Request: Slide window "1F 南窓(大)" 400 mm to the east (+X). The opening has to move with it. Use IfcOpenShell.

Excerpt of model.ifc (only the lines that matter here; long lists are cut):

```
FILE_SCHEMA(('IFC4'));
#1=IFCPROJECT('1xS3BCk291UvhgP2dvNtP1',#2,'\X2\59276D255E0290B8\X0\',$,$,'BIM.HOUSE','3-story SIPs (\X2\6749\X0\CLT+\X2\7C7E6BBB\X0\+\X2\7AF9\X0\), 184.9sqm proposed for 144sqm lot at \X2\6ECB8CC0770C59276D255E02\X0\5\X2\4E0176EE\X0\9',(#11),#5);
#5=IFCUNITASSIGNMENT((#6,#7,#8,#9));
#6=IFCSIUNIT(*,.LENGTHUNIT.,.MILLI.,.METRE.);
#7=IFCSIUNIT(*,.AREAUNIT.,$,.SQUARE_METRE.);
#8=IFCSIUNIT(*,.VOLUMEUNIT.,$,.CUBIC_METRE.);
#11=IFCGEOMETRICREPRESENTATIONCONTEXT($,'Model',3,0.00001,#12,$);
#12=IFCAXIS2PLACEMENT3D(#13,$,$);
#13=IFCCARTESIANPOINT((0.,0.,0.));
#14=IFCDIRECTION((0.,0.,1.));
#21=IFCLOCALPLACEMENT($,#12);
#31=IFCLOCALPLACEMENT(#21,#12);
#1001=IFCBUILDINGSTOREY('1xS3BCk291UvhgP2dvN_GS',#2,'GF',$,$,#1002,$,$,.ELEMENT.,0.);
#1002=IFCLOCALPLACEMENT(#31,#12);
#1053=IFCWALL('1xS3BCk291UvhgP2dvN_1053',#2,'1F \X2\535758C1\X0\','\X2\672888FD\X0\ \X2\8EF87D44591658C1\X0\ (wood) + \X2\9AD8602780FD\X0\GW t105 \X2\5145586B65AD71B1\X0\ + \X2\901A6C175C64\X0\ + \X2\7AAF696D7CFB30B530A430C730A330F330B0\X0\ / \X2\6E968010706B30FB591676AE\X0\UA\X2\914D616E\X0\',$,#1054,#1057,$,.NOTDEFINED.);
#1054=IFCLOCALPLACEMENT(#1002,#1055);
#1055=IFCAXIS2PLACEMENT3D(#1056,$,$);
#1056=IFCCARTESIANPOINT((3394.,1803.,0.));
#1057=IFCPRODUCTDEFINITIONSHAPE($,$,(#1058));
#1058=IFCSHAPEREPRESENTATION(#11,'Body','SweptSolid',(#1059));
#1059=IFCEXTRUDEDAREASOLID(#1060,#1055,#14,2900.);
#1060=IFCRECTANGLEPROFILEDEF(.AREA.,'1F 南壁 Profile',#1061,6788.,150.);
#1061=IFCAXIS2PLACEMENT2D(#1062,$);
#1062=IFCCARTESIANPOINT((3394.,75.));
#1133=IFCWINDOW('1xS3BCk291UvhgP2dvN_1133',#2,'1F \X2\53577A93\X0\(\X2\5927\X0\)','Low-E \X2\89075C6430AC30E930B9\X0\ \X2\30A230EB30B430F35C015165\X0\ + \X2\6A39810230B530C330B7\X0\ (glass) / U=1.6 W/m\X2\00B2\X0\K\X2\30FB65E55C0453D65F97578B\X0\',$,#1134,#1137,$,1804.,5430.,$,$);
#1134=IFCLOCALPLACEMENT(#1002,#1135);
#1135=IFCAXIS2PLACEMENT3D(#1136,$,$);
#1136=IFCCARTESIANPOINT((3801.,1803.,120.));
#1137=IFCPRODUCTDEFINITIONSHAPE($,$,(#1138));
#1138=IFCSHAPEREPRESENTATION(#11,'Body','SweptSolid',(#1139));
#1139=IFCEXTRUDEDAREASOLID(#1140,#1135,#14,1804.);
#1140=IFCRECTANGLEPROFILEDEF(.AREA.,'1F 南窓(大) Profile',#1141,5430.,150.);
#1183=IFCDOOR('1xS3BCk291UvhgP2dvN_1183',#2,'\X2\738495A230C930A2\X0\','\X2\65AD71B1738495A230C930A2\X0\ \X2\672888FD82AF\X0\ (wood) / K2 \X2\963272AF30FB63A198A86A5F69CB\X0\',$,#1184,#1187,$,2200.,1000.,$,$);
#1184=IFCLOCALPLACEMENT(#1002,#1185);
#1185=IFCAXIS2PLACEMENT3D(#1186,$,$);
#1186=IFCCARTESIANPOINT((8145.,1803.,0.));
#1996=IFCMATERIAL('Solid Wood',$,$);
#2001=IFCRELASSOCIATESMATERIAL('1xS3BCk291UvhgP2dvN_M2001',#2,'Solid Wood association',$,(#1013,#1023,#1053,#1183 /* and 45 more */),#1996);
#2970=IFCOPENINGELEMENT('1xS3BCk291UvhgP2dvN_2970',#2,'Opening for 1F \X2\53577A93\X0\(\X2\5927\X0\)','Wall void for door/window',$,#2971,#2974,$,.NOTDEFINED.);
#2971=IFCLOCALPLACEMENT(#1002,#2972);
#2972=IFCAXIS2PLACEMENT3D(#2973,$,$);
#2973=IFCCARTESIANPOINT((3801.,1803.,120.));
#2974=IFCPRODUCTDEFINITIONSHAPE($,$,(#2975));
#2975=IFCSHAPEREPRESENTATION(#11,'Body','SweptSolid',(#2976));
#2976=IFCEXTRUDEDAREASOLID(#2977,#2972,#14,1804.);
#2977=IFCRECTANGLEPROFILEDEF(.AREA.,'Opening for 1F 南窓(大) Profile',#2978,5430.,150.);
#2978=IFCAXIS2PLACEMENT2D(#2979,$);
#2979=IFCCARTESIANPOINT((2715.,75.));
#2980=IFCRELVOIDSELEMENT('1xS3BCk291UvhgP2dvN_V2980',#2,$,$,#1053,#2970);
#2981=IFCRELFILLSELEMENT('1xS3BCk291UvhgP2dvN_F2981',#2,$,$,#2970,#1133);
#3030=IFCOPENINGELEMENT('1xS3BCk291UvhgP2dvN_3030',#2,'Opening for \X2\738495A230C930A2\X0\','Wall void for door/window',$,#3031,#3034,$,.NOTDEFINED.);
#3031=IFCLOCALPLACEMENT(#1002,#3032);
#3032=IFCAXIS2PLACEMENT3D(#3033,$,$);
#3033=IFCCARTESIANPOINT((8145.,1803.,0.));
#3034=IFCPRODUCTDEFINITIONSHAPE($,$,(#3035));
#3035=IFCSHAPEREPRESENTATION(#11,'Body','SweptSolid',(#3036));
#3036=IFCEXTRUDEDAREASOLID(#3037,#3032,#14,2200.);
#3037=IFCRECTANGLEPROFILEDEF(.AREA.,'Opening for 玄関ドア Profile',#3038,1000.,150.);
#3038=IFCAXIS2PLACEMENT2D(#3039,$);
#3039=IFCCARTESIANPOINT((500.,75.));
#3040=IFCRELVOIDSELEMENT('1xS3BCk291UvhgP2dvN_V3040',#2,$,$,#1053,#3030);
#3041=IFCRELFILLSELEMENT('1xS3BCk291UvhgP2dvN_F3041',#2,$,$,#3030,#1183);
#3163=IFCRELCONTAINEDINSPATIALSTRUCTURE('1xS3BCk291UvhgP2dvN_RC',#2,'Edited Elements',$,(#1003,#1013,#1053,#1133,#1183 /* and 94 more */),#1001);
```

```python
import ifcopenshell
import ifcopenshell.api.geometry
import ifcopenshell.util.placement
import ifcopenshell.util.unit

model = ifcopenshell.open("model.ifc")
unit_scale = ifcopenshell.util.unit.calculate_unit_scale(model)

window = model.by_guid("1xS3BCk291UvhgP2dvN_1133")
opening = window.FillsVoids[0].RelatingOpeningElement
wall = opening.VoidsElements[0].RelatingBuildingElement

wall_matrix = ifcopenshell.util.placement.get_local_placement(wall.ObjectPlacement)
shift = wall_matrix[:3, 0] * 0.4 / unit_scale
before = ifcopenshell.util.placement.get_local_placement(window.ObjectPlacement)[:3, 3].copy()

# The window is not placed relative to its opening, so move both.
for product in (opening, window):
    matrix = ifcopenshell.util.placement.get_local_placement(product.ObjectPlacement)
    matrix[:3, 3] += shift
    ifcopenshell.api.geometry.edit_object_placement(model, product=product, matrix=matrix, is_si=False)

after = ifcopenshell.util.placement.get_local_placement(window.ObjectPlacement)[:3, 3]
print("window moved by", (after - before).round(3) + 0.0)

model.write("model-out.ifc")
```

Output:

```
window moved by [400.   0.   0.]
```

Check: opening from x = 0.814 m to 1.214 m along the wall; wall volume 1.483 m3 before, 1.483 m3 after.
